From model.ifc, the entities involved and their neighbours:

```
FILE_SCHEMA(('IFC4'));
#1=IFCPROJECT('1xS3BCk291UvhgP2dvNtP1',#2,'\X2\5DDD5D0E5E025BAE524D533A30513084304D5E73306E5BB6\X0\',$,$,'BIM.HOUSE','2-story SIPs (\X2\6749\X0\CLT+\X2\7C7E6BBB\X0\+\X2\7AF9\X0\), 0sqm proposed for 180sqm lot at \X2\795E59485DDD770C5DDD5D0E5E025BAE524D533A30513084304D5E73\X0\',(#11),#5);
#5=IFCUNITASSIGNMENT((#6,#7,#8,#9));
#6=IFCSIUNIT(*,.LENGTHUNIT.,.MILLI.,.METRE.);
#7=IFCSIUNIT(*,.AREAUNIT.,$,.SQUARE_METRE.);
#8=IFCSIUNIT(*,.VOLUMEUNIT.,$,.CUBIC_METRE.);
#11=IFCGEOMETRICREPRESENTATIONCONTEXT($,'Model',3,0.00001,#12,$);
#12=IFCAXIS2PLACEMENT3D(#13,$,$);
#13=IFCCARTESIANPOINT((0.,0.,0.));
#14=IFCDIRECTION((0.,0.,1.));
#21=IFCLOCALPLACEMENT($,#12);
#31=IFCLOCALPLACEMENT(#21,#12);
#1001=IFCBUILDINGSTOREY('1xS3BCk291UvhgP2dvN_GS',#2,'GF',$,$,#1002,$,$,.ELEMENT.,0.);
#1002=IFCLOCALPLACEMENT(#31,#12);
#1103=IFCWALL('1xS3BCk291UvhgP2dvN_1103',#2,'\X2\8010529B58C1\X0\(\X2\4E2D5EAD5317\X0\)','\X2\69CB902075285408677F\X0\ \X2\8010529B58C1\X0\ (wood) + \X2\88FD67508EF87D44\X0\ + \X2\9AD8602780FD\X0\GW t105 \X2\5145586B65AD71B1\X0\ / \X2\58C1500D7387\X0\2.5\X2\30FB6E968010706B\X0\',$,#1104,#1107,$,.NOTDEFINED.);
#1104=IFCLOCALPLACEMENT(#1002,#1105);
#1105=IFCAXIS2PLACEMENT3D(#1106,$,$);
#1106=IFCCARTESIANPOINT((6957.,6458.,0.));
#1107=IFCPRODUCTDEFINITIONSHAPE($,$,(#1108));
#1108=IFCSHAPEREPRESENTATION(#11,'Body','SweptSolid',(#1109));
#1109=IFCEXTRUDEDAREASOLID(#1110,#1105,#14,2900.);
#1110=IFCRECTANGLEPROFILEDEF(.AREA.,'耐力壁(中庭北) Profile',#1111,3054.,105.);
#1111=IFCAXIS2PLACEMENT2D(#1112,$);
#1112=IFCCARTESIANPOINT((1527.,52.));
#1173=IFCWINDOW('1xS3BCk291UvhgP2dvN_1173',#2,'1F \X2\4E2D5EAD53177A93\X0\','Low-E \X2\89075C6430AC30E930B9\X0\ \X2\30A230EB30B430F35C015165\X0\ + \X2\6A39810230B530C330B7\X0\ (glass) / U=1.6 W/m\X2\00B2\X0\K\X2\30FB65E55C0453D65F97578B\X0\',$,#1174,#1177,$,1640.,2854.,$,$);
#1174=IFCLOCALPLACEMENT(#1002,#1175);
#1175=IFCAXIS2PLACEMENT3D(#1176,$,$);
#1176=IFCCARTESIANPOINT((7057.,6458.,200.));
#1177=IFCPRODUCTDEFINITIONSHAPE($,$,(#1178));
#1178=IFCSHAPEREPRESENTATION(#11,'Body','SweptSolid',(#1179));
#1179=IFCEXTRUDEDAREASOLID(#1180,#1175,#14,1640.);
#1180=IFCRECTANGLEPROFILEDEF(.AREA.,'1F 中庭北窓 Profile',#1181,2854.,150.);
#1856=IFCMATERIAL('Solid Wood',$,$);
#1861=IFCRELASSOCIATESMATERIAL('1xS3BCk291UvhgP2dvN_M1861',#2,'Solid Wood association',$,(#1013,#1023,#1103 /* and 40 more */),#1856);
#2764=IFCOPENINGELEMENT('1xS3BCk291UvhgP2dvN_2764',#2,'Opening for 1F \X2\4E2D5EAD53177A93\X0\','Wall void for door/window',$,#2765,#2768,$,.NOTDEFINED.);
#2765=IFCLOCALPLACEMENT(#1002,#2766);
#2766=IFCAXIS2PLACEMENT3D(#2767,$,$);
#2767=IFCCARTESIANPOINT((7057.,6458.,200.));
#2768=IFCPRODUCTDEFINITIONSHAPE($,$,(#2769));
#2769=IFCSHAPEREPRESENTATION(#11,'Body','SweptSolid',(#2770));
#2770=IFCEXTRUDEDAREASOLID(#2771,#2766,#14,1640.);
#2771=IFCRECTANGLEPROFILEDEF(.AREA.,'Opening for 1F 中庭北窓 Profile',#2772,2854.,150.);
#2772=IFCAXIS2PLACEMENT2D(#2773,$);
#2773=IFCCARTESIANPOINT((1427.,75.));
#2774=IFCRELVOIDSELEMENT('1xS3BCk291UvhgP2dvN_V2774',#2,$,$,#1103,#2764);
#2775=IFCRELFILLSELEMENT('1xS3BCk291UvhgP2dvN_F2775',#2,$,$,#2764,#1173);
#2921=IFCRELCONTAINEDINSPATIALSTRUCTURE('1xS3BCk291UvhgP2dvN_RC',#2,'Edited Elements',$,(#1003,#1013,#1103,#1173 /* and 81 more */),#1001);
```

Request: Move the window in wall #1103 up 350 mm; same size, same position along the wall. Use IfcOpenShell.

```python
import numpy as np
import ifcopenshell
import ifcopenshell.api.geometry
import ifcopenshell.util.placement
import ifcopenshell.util.unit

model = ifcopenshell.open("model.ifc")
unit_scale = ifcopenshell.util.unit.calculate_unit_scale(model)

window = model.by_id(1173)
opening = window.FillsVoids[0].RelatingOpeningElement
dz = 350.0

shift = np.array([0.0, 0.0, dz])
# The window is not placed relative to its opening, so move both.
for product in (opening, window):
    matrix = ifcopenshell.util.placement.get_local_placement(product.ObjectPlacement)
    matrix[:3, 3] += shift
    ifcopenshell.api.geometry.edit_object_placement(model, product=product, matrix=matrix, is_si=False)

print(f"moved by {dz * unit_scale:+.3f} m")

model.write("model_v2.ifc")
```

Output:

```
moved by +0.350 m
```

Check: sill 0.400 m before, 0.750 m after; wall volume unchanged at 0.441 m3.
